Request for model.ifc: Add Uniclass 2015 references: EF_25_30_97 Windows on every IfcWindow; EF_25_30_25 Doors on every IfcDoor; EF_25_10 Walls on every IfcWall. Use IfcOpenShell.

First a look at what the model holds.

```python
import ifcopenshell

model = ifcopenshell.open("model.ifc")
print(model.schema)
print("classifications:", [c.Name for c in model.by_type("IfcClassification")])
for ifc_class in ("IfcDoor", "IfcRoof", "IfcStair", "IfcWall", "IfcWindow"):
    print(ifc_class, len(model.by_type(ifc_class)))
```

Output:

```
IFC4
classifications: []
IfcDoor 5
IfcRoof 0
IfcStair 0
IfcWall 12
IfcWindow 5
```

```python
import ifcopenshell
import ifcopenshell.api.classification

model = ifcopenshell.open("model.ifc")

system = ifcopenshell.api.classification.add_classification(model, classification="Uniclass 2015")

codes = {
    "IfcWindow": ("EF_25_30_97", "Windows"),
    "IfcDoor": ("EF_25_30_25", "Doors"),
    "IfcWall": ("EF_25_10", "Walls"),
}
for ifc_class, (code, name) in codes.items():
    products = model.by_type(ifc_class)
    ifcopenshell.api.classification.add_reference(
        model, products=products, classification=system, identification=code, name=name
    )
    print(code, len(products))

model.write("model_v2.ifc")
```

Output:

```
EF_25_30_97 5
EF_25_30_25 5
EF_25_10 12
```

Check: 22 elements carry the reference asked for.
